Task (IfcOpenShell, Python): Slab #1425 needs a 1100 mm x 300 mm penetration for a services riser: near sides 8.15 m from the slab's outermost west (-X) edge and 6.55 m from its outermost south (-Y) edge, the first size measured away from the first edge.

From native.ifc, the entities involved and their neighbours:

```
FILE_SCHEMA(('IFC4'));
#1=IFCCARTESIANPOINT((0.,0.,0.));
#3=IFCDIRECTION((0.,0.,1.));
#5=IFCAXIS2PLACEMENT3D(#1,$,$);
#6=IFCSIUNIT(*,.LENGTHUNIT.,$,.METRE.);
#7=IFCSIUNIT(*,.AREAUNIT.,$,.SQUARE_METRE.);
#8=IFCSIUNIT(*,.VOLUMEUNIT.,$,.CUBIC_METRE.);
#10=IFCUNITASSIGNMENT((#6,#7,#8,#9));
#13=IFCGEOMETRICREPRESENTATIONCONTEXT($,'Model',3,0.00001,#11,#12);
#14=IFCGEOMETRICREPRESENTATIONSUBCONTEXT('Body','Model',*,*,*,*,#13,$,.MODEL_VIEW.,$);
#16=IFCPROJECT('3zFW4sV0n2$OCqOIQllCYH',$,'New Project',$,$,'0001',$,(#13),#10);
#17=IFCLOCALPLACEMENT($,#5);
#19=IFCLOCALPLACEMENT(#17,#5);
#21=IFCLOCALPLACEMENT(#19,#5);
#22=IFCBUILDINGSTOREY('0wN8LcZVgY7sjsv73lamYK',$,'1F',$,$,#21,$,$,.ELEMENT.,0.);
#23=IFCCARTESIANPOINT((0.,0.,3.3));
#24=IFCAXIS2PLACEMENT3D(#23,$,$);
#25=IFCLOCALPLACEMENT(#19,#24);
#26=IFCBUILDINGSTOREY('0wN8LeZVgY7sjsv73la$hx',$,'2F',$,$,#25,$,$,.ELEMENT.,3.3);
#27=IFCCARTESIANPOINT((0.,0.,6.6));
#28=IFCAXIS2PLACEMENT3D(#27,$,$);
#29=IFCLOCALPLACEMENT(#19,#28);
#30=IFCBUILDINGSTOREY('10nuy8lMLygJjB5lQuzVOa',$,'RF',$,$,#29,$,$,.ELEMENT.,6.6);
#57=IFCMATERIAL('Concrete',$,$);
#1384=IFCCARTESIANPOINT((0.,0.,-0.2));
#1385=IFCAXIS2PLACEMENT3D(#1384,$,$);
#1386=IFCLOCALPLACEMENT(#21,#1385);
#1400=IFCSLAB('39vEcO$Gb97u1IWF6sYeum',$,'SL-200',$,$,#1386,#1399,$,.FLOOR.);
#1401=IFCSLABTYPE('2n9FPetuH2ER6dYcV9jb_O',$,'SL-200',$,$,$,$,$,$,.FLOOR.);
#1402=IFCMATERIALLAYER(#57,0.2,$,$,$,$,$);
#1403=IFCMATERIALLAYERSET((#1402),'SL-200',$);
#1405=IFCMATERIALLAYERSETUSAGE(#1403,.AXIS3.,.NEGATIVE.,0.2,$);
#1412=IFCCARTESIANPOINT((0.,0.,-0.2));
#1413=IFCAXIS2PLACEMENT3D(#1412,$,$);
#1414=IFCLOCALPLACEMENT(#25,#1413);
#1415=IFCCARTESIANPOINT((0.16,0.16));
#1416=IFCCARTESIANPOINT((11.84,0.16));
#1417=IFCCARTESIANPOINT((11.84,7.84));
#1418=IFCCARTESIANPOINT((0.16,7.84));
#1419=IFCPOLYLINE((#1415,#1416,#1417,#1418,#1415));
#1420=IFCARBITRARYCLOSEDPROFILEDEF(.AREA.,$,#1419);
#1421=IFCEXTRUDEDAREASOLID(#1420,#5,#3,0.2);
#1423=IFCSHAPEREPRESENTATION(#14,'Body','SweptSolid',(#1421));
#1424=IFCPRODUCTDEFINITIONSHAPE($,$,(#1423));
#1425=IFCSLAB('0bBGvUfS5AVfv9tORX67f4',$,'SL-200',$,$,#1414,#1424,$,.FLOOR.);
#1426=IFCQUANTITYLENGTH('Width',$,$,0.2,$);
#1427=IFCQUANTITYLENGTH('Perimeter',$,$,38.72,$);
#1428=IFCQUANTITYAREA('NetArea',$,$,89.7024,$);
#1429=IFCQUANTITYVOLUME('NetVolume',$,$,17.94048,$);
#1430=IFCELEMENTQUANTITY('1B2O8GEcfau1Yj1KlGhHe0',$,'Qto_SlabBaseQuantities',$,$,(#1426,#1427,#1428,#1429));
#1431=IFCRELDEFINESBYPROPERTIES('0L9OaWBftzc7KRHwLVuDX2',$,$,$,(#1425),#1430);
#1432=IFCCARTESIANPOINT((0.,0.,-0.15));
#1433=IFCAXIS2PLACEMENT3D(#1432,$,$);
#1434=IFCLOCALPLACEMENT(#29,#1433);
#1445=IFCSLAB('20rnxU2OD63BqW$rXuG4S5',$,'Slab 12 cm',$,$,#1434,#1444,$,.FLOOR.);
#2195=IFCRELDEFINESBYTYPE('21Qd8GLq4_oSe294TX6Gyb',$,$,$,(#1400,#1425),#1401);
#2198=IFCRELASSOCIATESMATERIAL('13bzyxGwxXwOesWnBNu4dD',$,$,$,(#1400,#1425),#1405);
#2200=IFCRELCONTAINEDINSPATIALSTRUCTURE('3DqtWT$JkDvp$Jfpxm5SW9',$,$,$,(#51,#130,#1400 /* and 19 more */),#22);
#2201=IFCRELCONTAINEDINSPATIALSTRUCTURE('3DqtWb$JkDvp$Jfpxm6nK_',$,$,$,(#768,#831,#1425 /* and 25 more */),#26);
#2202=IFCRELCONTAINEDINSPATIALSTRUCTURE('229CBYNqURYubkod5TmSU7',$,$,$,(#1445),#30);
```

```python
import numpy as np
import ifcopenshell
import ifcopenshell.api.feature
import ifcopenshell.api.geometry
import ifcopenshell.api.pset
import ifcopenshell.api.root
import ifcopenshell.geom
import ifcopenshell.util.element
import ifcopenshell.util.placement
import ifcopenshell.util.representation
import ifcopenshell.util.shape
import ifcopenshell.util.unit

model = ifcopenshell.open("native.ifc")
unit_scale = ifcopenshell.util.unit.calculate_unit_scale(model)
area_scale = ifcopenshell.util.unit.calculate_unit_scale(model, "AREAUNIT")
volume_scale = ifcopenshell.util.unit.calculate_unit_scale(model, "VOLUMEUNIT")
settings = ifcopenshell.geom.settings()


def volume(element):
    """Net volume in cubic metres, openings subtracted."""
    shape = ifcopenshell.geom.create_shape(settings, element)
    return ifcopenshell.util.shape.get_volume(shape.geometry)


slab = model.by_guid("0bBGvUfS5AVfv9tORX67f4")
before = volume(slab)

# Extent in the slab's own axes, in metres. The edges named are its -X and -Y sides.
slab_shape = ifcopenshell.geom.create_shape(settings, slab)
vertices = ifcopenshell.util.shape.get_vertices(slab_shape.geometry)
x_min, y_min, bottom = vertices.min(axis=0)
top = vertices[:, 2].max()

opening = ifcopenshell.api.root.create_entity(model, ifc_class="IfcOpeningElement", name="Services riser opening", predefined_type="OPENING")
context = ifcopenshell.util.representation.get_context(model, "Model", "Body", "MODEL_VIEW")
width, depth = 1.1, 0.3
outline = [(0.0, 0.0), (width, 0.0), (width, depth), (0.0, depth), (0.0, 0.0)]
# Overshoot both faces by 50 mm so the cut is clean.
shape = ifcopenshell.api.geometry.add_slab_representation(
    model, context=context, depth=top - bottom + 0.1, polyline=outline
)
ifcopenshell.api.geometry.assign_representation(model, product=opening, representation=shape)

matrix = ifcopenshell.util.placement.get_local_placement(slab.ObjectPlacement)
matrix[:, 3] = matrix @ np.append(np.array([x_min + 8.15, y_min + 6.55, bottom - 0.05]) / unit_scale, 1.0)
ifcopenshell.api.geometry.edit_object_placement(model, product=opening, matrix=matrix, is_si=False)
ifcopenshell.api.feature.add_feature(model, feature=opening, element=slab)

after = volume(slab)

# Update the slab's stored quantities.
qto = model.by_id(ifcopenshell.util.element.get_pset(slab, "Qto_SlabBaseQuantities", should_inherit=False)["id"])
ifcopenshell.api.pset.edit_qto(model, qto=qto, properties={
    "NetArea": after / (top - bottom) / area_scale,
    "NetVolume": after / volume_scale,
})

print(f"slab volume {before:.3f} -> {after:.3f} m3")

model.write("native_rev.ifc")
```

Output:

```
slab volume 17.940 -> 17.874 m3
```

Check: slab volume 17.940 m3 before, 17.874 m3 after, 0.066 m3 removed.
